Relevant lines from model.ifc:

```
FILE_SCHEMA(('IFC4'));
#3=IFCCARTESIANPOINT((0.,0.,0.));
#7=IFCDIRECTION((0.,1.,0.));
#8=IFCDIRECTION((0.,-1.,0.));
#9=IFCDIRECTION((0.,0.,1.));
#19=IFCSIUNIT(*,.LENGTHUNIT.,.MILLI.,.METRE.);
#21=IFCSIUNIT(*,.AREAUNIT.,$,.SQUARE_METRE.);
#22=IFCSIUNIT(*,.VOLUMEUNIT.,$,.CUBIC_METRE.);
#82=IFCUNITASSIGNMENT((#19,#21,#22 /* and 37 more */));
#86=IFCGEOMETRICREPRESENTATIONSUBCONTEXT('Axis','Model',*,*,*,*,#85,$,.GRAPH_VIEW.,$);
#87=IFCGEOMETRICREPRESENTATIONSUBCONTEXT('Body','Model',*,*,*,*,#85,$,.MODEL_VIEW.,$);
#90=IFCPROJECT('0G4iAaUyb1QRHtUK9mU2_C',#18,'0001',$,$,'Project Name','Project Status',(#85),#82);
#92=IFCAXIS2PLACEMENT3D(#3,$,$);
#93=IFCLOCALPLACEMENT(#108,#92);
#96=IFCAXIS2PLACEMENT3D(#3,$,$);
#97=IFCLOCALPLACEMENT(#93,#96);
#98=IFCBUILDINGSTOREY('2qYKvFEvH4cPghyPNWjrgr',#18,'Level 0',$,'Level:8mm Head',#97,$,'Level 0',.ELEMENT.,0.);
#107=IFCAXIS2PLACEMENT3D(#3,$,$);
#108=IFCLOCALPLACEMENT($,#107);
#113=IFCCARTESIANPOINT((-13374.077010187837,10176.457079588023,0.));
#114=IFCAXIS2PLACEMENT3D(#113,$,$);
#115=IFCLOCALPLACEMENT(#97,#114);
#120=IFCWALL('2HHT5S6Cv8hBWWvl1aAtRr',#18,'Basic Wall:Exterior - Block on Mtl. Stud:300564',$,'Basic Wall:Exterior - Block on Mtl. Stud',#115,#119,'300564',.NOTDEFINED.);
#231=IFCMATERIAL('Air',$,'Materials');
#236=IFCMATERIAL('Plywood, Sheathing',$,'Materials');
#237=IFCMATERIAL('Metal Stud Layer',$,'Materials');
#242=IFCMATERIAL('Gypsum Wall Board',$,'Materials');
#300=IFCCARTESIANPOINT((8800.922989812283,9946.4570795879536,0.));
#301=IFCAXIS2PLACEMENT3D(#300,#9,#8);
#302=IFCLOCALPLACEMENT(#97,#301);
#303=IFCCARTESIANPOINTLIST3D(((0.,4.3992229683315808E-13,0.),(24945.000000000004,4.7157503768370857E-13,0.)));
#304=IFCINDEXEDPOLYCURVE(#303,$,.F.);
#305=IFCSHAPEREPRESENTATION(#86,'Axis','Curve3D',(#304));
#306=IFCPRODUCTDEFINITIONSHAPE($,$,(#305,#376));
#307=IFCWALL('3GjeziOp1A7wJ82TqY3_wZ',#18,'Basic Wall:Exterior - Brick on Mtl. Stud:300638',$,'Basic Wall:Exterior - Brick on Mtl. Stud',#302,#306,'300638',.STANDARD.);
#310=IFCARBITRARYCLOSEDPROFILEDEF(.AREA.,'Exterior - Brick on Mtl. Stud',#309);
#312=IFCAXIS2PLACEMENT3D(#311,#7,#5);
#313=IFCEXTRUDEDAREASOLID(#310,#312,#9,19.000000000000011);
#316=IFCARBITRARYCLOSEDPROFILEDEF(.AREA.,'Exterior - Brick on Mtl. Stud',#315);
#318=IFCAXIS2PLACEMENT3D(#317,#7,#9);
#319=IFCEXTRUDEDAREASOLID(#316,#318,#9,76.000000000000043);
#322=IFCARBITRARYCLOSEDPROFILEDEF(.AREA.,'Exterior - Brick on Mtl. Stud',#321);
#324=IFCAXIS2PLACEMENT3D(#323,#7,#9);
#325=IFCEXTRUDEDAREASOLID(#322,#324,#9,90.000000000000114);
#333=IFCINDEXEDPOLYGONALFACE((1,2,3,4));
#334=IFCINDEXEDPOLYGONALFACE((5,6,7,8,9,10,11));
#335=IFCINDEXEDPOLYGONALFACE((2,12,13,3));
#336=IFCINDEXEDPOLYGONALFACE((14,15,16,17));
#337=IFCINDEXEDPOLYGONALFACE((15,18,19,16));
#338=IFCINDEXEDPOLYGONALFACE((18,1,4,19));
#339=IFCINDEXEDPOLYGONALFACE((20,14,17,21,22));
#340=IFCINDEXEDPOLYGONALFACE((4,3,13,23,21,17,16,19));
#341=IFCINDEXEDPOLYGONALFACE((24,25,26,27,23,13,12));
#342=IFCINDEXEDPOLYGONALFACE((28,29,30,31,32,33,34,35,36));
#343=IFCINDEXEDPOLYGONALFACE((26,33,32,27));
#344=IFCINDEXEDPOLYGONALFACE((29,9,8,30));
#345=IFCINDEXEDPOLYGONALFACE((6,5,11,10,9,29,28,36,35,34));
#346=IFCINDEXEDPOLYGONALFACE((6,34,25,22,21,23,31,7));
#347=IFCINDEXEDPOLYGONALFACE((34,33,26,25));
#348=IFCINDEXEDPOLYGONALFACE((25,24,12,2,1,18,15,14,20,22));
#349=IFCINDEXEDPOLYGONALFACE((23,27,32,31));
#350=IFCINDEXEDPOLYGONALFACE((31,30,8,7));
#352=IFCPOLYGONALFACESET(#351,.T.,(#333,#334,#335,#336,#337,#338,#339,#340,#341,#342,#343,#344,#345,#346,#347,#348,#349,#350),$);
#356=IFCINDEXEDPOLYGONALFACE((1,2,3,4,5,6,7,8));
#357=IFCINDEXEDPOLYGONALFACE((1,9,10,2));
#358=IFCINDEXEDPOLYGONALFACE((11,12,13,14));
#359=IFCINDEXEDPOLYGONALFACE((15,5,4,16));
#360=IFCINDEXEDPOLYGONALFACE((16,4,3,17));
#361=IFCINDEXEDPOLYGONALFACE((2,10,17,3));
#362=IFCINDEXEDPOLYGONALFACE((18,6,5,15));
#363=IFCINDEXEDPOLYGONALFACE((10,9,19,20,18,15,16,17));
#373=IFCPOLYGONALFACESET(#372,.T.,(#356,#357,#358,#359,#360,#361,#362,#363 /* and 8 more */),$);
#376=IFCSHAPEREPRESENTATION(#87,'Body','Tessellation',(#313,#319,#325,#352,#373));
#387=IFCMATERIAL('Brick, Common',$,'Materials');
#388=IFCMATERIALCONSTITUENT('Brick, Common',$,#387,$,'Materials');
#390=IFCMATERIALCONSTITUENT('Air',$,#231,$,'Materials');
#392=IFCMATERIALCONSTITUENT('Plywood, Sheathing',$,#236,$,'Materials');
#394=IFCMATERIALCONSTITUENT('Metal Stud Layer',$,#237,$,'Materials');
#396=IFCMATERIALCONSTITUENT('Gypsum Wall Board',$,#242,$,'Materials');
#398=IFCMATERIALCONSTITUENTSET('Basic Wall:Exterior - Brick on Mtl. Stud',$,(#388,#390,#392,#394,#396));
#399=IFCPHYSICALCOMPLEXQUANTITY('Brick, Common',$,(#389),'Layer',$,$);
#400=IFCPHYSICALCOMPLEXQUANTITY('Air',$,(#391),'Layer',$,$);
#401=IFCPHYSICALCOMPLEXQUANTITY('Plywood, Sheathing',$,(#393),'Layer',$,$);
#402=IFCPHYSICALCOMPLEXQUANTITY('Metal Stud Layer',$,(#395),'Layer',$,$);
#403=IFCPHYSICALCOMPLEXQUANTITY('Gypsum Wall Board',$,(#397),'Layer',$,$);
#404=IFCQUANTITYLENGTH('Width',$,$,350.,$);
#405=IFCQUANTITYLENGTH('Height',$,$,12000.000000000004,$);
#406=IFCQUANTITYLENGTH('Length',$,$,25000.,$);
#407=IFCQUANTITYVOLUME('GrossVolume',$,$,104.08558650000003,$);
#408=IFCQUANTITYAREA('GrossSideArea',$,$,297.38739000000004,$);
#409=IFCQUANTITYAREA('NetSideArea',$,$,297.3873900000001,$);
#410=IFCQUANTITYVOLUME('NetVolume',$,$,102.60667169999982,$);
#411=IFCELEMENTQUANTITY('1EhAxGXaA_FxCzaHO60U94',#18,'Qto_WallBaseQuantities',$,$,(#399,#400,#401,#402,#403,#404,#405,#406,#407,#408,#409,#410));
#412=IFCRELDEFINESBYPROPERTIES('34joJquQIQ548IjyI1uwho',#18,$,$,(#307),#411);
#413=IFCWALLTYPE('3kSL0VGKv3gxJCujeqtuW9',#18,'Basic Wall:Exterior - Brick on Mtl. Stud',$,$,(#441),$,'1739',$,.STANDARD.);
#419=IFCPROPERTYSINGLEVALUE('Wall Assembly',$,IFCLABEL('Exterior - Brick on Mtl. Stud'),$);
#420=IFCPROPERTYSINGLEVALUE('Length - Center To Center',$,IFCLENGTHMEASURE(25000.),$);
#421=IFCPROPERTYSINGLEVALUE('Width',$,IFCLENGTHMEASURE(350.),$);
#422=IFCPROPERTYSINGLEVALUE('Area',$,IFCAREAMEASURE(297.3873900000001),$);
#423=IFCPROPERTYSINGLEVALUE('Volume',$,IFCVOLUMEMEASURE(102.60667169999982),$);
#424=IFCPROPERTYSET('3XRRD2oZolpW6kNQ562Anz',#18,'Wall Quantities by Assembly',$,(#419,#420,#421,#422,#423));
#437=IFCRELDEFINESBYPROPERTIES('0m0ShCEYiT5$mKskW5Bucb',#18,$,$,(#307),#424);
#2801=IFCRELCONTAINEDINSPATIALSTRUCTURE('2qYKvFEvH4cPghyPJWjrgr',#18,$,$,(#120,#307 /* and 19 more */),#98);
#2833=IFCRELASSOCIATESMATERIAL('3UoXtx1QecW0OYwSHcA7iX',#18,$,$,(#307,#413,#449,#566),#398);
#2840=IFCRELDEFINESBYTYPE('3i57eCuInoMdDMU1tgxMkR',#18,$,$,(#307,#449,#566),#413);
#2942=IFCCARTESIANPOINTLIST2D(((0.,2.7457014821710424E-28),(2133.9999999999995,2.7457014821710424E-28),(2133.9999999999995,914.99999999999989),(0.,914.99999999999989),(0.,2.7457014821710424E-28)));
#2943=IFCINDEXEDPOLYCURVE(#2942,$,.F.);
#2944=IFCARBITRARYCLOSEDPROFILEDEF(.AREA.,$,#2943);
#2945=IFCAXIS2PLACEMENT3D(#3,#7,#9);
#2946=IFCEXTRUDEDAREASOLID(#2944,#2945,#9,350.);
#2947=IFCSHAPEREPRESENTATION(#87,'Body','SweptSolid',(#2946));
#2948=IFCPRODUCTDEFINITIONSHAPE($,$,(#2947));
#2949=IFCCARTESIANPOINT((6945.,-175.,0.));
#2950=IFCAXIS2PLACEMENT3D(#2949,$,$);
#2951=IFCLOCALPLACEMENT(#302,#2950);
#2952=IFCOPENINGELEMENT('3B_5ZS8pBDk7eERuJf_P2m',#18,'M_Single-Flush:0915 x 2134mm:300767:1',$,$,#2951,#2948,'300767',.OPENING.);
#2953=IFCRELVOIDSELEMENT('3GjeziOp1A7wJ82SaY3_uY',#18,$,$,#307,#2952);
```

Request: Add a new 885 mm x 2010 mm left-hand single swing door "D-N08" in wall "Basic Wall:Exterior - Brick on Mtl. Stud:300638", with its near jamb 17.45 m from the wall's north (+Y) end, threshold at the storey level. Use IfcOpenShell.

```python
import numpy as np
import ifcopenshell
import ifcopenshell.api.feature
import ifcopenshell.api.geometry
import ifcopenshell.api.pset
import ifcopenshell.api.root
import ifcopenshell.api.spatial
import ifcopenshell.geom
import ifcopenshell.util.element
import ifcopenshell.util.placement
import ifcopenshell.util.representation
import ifcopenshell.util.shape
import ifcopenshell.util.unit

model = ifcopenshell.open("model.ifc")
unit_scale = ifcopenshell.util.unit.calculate_unit_scale(model)
area_scale = ifcopenshell.util.unit.calculate_unit_scale(model, "AREAUNIT")
volume_scale = ifcopenshell.util.unit.calculate_unit_scale(model, "VOLUMEUNIT")
settings = ifcopenshell.geom.settings()


def volume(element):
    """Net volume in cubic metres, openings subtracted."""
    shape = ifcopenshell.geom.create_shape(settings, element)
    return ifcopenshell.util.shape.get_volume(shape.geometry)


wall = model.by_guid("3GjeziOp1A7wJ82TqY3_wZ")
storey = ifcopenshell.util.element.get_container(wall, ifc_class="IfcBuildingStorey")
context = ifcopenshell.util.representation.get_context(model, "Model", "Body", "MODEL_VIEW")
before = volume(wall)

width, height, from_end, sill = 0.885, 2.01, 17.45, 0.0  # metres

# The wall runs along its own X axis, and the end named is its -X end.
wall_shape = ifcopenshell.geom.create_shape(settings, wall)
x, y, z = ifcopenshell.util.shape.get_vertices(wall_shape.geometry).T
start = x.min() + from_end
face, thickness = float(y.min()), float(y.max() - y.min())
wall_matrix = ifcopenshell.util.placement.get_local_placement(wall.ObjectPlacement)
level = ifcopenshell.util.placement.get_local_placement(storey.ObjectPlacement)[2, 3]


def in_wall(x, y):
    """Placement at x, y metres in the wall's axes, at sill height."""
    matrix = wall_matrix.copy()
    matrix[:, 3] = wall_matrix @ np.array([x / unit_scale, y / unit_scale, 0.0, 1.0])
    matrix[2, 3] = level + sill / unit_scale
    return matrix


# Opening: a box that overshoots both wall faces by 50 mm.
opening = ifcopenshell.api.root.create_entity(model, ifc_class="IfcOpeningElement", predefined_type="OPENING")
box = ifcopenshell.api.geometry.add_wall_representation(
    model, context=context, length=width, height=height, thickness=thickness + 0.1
)
ifcopenshell.api.geometry.assign_representation(model, product=opening, representation=box)
ifcopenshell.api.geometry.edit_object_placement(model, product=opening, matrix=in_wall(start, face - 0.05), is_si=False)
ifcopenshell.api.feature.add_feature(model, feature=opening, element=wall)

door = ifcopenshell.api.root.create_entity(model, ifc_class="IfcDoor", name="D-N08", predefined_type="DOOR")
door.OverallWidth, door.OverallHeight = width / unit_scale, height / unit_scale
door.OperationType = "SINGLE_SWING_LEFT"
body = ifcopenshell.api.geometry.add_door_representation(
    model,
    context=context,
    overall_width=door.OverallWidth,
    overall_height=door.OverallHeight,
    operation_type="SINGLE_SWING_LEFT",
    lining_properties={"LiningDepth": thickness / unit_scale, "ThresholdDepth": thickness / unit_scale},
)
ifcopenshell.api.geometry.assign_representation(model, product=door, representation=body)
ifcopenshell.api.spatial.assign_container(model, products=[door], relating_structure=storey)
ifcopenshell.api.feature.add_filling(model, opening=opening, element=door)

# The lining spans the wall, so the door starts at the wall face.
ifcopenshell.api.geometry.edit_object_placement(model, product=door, matrix=in_wall(start, face), is_si=False)

after = volume(wall)

# Update the wall's stored quantities.
qto = model.by_id(ifcopenshell.util.element.get_pset(wall, "Qto_WallBaseQuantities", should_inherit=False)["id"])
ifcopenshell.api.pset.edit_qto(model, qto=qto, properties={
    "NetSideArea": after / thickness / area_scale,
    "NetVolume": after / volume_scale,
})
pset = model.by_id(ifcopenshell.util.element.get_pset(wall, "Wall Quantities by Assembly", should_inherit=False)["id"])
ifcopenshell.api.pset.edit_pset(model, pset=pset, properties={
    "Area": model.create_entity("IfcAreaMeasure", after / thickness / area_scale),
    "Volume": model.create_entity("IfcVolumeMeasure", after / volume_scale),
})

print(f"wall volume {before:.3f} -> {after:.3f} m3")

model.write("model_v2.ifc")
```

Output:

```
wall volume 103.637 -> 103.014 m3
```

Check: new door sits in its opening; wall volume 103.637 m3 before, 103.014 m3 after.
